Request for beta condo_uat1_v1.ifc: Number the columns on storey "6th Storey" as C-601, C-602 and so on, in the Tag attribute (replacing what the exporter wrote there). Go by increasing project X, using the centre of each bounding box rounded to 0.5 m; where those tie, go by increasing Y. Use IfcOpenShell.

First a look at what the model holds.

```python
import ifcopenshell
import ifcopenshell.util.element
import ifcopenshell.util.placement

model = ifcopenshell.open("beta condo_uat1_v1.ifc")
print(model.schema)
storey = next(s for s in model.by_type("IfcBuildingStorey") if s.Name == "6th Storey")
columns = [e for e in ifcopenshell.util.element.get_decomposition(storey) if e.is_a("IfcColumn")]
for e in sorted(columns, key=lambda e: e.id()):
    origin = ifcopenshell.util.placement.get_local_placement(e.ObjectPlacement)[:3, 3]
    print(e.id(), e.Tag, e.Name, origin.round(2) + 0.0, sep=" | ")
```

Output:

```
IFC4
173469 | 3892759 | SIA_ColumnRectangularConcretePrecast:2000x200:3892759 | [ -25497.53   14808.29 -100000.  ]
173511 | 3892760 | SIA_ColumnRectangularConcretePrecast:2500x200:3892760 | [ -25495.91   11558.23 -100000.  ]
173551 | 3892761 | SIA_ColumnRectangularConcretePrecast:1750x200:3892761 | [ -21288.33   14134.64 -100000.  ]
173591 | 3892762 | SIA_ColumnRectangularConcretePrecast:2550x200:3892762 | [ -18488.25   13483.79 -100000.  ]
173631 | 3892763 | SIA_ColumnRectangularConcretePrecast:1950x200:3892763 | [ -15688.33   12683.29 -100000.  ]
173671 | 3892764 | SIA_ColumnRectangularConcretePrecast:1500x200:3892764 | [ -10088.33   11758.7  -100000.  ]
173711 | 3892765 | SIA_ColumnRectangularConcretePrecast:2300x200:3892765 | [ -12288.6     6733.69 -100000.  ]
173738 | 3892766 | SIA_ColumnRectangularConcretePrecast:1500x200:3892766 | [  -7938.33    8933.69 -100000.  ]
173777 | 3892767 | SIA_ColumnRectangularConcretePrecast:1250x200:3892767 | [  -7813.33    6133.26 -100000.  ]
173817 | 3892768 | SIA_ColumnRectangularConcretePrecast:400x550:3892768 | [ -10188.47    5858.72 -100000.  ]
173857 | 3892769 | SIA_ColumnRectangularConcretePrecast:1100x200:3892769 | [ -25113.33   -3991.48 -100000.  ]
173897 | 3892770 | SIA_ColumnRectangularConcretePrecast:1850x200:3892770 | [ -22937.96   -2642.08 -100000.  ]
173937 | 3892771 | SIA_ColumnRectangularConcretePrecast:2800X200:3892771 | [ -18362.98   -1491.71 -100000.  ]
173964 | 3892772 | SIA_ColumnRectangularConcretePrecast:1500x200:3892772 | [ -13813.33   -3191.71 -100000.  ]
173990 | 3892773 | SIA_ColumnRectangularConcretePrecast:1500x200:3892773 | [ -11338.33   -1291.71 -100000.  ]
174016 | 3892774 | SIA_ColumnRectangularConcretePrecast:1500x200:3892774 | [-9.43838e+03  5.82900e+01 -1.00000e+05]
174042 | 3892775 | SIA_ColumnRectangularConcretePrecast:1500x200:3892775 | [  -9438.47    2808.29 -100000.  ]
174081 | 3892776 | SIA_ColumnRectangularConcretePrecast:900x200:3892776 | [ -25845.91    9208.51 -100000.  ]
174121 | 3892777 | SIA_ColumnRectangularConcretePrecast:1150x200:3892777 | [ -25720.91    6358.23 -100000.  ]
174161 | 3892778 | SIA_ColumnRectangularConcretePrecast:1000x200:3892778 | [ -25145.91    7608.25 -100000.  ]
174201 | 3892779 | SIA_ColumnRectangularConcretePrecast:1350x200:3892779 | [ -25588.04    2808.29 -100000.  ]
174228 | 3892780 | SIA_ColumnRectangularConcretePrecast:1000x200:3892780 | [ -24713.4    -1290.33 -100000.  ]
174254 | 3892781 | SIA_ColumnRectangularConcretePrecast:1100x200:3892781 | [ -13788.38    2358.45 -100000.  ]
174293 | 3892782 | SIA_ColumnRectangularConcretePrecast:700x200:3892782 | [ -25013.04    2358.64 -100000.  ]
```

```python
import ifcopenshell
import ifcopenshell.geom
import ifcopenshell.util.element
import ifcopenshell.util.shape

model = ifcopenshell.open("beta condo_uat1_v1.ifc")
settings = ifcopenshell.geom.settings()
settings.set("use-world-coords", True)


def centre(element):
    shape = ifcopenshell.geom.create_shape(settings, element)
    return ifcopenshell.util.shape.get_bbox_centroid(shape.geometry)


storey = next(s for s in model.by_type("IfcBuildingStorey") if s.Name == "6th Storey")
columns = [e for e in ifcopenshell.util.element.get_decomposition(storey) if e.is_a("IfcColumn")]

# Insertion points can sit at a corner or the storey origin, so sort by the geometry (in metres).
centres = {e: centre(e) for e in columns}
columns.sort(key=lambda e: (round(centres[e][0] / 0.5), centres[e][1]))

for i, e in enumerate(columns, start=1):
    number = f"C-6{i:02d}"
    e.Tag = number
    print(e.id(), number)

model.write("beta condo_uat1_v1_updated.ifc")
```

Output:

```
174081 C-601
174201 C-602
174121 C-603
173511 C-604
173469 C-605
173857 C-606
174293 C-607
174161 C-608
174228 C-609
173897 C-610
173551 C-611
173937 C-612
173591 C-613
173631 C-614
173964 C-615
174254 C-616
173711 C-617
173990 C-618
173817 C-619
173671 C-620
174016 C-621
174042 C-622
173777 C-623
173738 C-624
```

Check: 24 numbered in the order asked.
